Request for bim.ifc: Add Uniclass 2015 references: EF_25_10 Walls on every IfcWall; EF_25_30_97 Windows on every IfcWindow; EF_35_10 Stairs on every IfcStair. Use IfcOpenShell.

First a look at what the model holds.

```python
import ifcopenshell

model = ifcopenshell.open("bim.ifc")
print(model.schema)
print("classifications:", [c.Name for c in model.by_type("IfcClassification")])
for ifc_class in ("IfcDoor", "IfcRoof", "IfcStair", "IfcWall", "IfcWindow"):
    print(ifc_class, len(model.by_type(ifc_class)))
```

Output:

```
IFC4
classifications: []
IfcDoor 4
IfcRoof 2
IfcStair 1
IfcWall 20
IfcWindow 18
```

```python
import ifcopenshell
import ifcopenshell.api.classification

model = ifcopenshell.open("bim.ifc")

system = ifcopenshell.api.classification.add_classification(model, classification="Uniclass 2015")

codes = {
    "IfcWall": ("EF_25_10", "Walls"),
    "IfcWindow": ("EF_25_30_97", "Windows"),
    "IfcStair": ("EF_35_10", "Stairs"),
}
for ifc_class, (code, name) in codes.items():
    products = model.by_type(ifc_class)
    ifcopenshell.api.classification.add_reference(
        model, products=products, classification=system, identification=code, name=name
    )
    print(code, len(products))

model.write("bim-out.ifc")
```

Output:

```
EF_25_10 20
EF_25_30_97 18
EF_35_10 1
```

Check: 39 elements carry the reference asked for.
